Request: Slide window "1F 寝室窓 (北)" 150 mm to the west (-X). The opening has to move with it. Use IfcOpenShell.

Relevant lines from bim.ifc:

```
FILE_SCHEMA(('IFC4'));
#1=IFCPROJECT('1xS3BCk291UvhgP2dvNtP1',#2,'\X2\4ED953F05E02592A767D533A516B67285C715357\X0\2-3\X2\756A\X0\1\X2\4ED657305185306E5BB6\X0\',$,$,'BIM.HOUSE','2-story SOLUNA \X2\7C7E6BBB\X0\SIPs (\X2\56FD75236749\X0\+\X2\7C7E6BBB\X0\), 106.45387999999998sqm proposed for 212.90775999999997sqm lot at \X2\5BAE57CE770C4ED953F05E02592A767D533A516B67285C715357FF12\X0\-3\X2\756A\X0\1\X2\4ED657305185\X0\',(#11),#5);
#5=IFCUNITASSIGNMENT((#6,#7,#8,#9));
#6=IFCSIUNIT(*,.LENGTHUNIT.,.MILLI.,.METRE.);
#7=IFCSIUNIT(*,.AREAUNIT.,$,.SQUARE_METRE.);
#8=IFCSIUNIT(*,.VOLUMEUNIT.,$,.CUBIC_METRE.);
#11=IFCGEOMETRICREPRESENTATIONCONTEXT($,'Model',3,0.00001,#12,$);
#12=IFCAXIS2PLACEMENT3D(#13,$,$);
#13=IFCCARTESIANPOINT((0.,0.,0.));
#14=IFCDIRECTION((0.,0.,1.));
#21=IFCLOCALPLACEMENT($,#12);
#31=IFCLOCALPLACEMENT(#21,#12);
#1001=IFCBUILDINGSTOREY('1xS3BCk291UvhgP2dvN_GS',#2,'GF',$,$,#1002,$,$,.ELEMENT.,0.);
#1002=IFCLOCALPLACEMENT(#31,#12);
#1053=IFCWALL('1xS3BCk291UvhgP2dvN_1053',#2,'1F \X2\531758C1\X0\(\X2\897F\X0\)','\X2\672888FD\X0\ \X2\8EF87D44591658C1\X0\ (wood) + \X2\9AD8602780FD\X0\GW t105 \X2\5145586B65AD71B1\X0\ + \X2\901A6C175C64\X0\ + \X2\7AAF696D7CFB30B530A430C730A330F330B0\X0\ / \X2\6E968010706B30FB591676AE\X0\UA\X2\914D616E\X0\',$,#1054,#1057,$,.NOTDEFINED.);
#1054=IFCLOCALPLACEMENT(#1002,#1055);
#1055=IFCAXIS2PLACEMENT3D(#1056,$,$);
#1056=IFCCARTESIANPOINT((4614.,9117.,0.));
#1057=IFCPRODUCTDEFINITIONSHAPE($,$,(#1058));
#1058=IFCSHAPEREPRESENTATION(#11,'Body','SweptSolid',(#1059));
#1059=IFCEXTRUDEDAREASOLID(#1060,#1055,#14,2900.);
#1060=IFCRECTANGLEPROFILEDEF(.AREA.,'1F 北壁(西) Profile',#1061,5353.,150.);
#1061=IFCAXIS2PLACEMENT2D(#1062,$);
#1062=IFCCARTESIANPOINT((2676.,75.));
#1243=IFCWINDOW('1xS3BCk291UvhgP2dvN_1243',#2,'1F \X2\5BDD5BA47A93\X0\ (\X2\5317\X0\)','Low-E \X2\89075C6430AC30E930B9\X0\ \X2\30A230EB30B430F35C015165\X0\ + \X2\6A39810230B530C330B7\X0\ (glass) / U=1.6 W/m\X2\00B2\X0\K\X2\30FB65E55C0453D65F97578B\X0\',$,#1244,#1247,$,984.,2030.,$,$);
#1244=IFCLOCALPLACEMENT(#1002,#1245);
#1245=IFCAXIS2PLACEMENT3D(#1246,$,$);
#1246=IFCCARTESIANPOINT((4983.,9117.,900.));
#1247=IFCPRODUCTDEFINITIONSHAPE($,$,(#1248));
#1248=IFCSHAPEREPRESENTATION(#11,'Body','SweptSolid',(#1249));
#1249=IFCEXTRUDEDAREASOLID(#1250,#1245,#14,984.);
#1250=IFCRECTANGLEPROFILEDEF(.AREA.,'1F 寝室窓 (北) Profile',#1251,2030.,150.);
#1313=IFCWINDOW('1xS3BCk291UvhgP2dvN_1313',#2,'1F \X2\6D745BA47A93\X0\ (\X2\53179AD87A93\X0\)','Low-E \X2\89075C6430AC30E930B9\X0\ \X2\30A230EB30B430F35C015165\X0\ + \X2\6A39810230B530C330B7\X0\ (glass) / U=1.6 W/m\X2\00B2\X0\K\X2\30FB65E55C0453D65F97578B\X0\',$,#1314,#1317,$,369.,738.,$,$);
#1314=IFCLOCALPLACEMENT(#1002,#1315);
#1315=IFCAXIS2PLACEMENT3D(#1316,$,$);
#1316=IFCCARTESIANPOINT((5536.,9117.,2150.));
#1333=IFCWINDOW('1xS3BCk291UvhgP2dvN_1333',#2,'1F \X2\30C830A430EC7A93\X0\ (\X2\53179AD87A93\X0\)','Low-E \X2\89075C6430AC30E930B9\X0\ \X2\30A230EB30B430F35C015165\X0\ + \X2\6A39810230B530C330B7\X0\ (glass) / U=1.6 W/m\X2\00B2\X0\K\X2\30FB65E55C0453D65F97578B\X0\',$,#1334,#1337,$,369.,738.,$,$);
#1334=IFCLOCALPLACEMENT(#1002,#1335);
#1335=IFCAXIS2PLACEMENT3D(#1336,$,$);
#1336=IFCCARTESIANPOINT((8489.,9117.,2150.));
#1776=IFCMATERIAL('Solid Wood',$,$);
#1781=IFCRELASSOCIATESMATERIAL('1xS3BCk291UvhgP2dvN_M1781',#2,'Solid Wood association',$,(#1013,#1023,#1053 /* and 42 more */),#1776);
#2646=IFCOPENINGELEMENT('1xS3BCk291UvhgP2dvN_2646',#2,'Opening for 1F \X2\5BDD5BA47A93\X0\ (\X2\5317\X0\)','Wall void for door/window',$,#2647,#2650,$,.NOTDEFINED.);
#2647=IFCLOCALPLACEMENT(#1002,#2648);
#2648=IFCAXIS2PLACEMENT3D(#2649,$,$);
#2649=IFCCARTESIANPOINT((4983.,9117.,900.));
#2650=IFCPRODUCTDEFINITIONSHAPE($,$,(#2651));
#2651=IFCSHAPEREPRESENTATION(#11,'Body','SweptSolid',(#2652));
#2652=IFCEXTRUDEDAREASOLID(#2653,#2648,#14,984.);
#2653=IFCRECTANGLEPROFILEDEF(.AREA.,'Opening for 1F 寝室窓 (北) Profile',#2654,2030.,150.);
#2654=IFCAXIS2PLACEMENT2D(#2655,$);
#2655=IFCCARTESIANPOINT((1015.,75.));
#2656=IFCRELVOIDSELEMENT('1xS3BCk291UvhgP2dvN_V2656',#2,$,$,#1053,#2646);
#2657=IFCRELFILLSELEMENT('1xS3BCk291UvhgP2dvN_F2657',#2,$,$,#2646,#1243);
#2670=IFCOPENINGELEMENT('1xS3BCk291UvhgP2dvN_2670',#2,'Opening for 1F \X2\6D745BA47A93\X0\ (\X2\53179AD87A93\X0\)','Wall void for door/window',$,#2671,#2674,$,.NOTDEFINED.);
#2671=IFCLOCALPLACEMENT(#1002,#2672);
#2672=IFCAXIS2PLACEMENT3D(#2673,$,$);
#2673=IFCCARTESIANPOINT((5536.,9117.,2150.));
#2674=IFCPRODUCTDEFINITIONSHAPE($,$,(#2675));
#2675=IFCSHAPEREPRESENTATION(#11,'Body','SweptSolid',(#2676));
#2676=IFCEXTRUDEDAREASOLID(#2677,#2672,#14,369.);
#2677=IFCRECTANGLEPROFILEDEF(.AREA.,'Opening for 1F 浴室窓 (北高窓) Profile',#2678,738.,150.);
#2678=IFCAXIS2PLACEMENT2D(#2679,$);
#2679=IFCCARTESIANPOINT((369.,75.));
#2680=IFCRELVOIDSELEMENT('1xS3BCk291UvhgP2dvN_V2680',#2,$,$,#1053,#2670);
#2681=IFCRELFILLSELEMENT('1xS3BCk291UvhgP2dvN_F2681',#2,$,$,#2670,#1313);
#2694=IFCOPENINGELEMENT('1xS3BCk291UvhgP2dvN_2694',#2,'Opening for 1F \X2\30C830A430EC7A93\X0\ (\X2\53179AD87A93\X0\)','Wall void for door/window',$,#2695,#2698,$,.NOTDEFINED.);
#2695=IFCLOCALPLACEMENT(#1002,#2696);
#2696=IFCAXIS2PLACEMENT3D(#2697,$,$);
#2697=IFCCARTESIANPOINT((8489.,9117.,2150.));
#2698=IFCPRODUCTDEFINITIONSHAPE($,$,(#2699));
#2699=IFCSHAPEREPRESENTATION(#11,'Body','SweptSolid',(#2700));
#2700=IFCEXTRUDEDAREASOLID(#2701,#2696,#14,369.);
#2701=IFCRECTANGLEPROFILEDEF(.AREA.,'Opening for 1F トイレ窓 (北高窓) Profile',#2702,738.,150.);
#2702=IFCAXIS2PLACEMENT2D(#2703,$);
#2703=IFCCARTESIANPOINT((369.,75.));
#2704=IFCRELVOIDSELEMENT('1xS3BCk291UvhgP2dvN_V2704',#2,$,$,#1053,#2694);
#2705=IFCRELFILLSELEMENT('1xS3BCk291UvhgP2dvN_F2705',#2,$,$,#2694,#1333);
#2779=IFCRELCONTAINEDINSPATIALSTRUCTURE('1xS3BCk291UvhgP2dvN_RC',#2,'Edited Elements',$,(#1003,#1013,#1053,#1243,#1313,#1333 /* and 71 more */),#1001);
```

```python
import ifcopenshell
import ifcopenshell.api.geometry
import ifcopenshell.util.placement
import ifcopenshell.util.unit

model = ifcopenshell.open("bim.ifc")
unit_scale = ifcopenshell.util.unit.calculate_unit_scale(model)

window = model.by_guid("1xS3BCk291UvhgP2dvN_1243")
opening = window.FillsVoids[0].RelatingOpeningElement
wall = opening.VoidsElements[0].RelatingBuildingElement

wall_matrix = ifcopenshell.util.placement.get_local_placement(wall.ObjectPlacement)
shift = wall_matrix[:3, 0] * -0.15 / unit_scale
before = ifcopenshell.util.placement.get_local_placement(window.ObjectPlacement)[:3, 3].copy()

# The window is not placed relative to its opening, so move both.
for product in (opening, window):
    matrix = ifcopenshell.util.placement.get_local_placement(product.ObjectPlacement)
    matrix[:3, 3] += shift
    ifcopenshell.api.geometry.edit_object_placement(model, product=product, matrix=matrix, is_si=False)

after = ifcopenshell.util.placement.get_local_placement(window.ObjectPlacement)[:3, 3]
print("window moved by", (after - before).round(3) + 0.0)

model.write("bim_rev.ifc")
```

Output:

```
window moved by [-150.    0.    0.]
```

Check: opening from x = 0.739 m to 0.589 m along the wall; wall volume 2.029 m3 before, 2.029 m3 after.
